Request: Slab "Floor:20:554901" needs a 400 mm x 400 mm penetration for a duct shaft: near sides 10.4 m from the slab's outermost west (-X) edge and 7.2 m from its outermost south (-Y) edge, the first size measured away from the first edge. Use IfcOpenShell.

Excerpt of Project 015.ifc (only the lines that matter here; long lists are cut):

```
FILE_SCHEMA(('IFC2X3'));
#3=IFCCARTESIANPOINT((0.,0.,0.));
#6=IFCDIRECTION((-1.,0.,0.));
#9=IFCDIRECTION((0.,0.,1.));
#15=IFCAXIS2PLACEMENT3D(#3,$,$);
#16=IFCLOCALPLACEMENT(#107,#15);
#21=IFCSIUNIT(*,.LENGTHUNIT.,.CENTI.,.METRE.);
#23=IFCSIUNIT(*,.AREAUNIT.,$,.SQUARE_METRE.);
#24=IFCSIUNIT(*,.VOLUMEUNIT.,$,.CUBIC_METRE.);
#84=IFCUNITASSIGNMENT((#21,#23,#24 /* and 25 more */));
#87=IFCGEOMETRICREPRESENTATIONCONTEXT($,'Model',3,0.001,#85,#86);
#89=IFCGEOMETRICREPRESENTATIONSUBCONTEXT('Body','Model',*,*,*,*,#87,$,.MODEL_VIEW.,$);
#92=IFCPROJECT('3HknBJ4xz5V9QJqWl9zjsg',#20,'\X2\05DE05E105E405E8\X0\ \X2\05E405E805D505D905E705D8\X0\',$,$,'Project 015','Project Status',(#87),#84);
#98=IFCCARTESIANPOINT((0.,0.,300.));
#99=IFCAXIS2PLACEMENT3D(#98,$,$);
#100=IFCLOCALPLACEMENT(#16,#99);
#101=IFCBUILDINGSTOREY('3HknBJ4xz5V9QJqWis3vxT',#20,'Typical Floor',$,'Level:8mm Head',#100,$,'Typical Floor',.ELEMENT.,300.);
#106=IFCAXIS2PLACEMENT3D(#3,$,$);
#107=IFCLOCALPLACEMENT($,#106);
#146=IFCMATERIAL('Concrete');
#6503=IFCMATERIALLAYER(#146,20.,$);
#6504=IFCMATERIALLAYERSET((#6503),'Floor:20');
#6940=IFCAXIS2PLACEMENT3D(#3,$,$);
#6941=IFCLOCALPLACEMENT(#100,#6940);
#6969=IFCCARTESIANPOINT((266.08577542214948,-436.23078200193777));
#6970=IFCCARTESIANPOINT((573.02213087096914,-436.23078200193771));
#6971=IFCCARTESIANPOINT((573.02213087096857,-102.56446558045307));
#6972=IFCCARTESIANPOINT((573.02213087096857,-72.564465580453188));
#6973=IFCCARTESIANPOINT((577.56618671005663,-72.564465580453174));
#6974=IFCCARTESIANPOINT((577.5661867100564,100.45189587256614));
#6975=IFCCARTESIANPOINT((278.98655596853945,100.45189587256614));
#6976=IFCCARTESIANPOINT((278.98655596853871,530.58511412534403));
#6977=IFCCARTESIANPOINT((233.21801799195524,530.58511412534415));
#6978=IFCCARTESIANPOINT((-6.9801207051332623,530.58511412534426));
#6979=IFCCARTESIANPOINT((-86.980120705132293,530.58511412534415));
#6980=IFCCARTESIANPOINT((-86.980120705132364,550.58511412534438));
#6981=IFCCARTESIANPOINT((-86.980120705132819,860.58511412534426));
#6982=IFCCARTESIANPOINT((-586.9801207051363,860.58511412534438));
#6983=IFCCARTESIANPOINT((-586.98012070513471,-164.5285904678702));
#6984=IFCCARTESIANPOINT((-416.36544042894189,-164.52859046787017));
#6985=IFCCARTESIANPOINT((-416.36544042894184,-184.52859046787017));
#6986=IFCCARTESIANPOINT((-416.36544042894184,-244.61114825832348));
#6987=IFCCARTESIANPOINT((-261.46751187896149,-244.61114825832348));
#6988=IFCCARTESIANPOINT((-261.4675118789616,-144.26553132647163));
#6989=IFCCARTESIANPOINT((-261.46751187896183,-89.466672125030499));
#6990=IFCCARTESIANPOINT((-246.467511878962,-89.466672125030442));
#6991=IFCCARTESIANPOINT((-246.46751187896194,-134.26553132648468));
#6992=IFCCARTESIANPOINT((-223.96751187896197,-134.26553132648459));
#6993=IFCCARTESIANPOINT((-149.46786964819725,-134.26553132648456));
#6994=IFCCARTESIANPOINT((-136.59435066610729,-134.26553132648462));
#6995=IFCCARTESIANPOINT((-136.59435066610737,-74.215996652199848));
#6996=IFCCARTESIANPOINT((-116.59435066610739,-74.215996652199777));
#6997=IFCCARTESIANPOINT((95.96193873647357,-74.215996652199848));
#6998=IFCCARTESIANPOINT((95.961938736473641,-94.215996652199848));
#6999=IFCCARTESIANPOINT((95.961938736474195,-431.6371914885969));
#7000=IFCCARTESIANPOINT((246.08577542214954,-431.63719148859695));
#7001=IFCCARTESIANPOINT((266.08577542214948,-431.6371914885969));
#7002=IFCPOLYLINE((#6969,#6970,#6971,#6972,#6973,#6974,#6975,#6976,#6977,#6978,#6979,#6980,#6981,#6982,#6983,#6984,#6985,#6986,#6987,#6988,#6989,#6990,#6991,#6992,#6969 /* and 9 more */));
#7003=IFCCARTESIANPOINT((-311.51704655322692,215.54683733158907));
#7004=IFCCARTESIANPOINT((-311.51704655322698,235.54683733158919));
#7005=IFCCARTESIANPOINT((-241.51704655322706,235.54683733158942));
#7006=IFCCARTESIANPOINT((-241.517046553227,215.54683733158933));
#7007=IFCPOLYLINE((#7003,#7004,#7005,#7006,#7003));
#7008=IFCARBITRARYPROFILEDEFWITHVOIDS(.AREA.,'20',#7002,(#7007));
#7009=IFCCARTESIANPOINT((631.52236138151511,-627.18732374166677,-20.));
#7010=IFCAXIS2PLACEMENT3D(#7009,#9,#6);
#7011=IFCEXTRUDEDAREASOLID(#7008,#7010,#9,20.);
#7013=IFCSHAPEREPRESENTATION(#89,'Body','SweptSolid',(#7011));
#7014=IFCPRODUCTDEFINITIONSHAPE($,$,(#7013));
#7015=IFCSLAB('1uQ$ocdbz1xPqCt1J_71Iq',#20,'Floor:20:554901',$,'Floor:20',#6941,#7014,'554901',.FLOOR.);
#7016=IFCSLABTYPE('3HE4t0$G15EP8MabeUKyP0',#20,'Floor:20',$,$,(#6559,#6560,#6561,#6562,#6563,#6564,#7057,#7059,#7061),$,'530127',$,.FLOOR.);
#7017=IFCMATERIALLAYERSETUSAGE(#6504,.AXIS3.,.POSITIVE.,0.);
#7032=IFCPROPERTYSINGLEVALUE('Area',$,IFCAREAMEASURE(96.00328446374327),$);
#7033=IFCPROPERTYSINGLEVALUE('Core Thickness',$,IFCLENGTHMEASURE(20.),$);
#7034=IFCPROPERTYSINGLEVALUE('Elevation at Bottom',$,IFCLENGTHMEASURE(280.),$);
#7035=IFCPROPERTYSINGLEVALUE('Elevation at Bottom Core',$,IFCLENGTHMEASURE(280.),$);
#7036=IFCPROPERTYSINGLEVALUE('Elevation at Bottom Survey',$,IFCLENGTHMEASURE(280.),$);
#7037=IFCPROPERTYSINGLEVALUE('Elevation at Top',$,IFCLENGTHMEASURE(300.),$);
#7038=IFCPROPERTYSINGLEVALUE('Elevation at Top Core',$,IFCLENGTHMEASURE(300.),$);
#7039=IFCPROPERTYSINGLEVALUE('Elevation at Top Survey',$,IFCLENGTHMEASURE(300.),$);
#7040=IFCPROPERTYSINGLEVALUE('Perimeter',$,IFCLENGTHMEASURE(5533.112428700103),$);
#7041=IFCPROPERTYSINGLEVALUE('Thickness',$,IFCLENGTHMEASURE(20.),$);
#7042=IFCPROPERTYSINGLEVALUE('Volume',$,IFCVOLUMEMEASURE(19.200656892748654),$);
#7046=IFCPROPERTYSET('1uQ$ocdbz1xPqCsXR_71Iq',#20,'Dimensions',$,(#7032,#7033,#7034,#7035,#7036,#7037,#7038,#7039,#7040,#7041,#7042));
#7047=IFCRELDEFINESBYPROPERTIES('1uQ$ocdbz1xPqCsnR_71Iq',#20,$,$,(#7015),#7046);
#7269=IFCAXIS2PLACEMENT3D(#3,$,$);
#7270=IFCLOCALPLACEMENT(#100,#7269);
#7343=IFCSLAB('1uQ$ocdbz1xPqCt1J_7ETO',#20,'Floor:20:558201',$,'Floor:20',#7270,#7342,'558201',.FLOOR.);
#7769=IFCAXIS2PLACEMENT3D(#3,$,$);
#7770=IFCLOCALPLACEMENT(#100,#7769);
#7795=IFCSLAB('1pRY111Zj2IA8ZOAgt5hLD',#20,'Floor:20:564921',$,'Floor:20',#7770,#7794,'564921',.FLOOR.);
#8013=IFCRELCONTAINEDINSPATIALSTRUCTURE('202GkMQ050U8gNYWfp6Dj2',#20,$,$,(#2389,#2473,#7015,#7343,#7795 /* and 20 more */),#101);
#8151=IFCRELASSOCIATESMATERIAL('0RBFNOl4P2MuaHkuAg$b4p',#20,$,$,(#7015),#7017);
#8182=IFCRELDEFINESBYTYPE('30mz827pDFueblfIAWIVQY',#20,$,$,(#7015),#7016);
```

```python
import numpy as np
import ifcopenshell
import ifcopenshell.api.feature
import ifcopenshell.api.geometry
import ifcopenshell.api.pset
import ifcopenshell.api.root
import ifcopenshell.geom
import ifcopenshell.util.element
import ifcopenshell.util.placement
import ifcopenshell.util.representation
import ifcopenshell.util.shape
import ifcopenshell.util.unit

model = ifcopenshell.open("Project 015.ifc")
unit_scale = ifcopenshell.util.unit.calculate_unit_scale(model)
area_scale = ifcopenshell.util.unit.calculate_unit_scale(model, "AREAUNIT")
volume_scale = ifcopenshell.util.unit.calculate_unit_scale(model, "VOLUMEUNIT")
settings = ifcopenshell.geom.settings()


def volume(element):
    """Net volume in cubic metres, openings subtracted."""
    shape = ifcopenshell.geom.create_shape(settings, element)
    return ifcopenshell.util.shape.get_volume(shape.geometry)


slab = model.by_id(7015)
before = volume(slab)

# Extent in the slab's own axes, in metres. The edges named are its -X and -Y sides.
slab_shape = ifcopenshell.geom.create_shape(settings, slab)
vertices = ifcopenshell.util.shape.get_vertices(slab_shape.geometry)
x_min, y_min, bottom = vertices.min(axis=0)
top = vertices[:, 2].max()

opening = ifcopenshell.api.root.create_entity(model, ifc_class="IfcOpeningElement", name="Duct shaft opening")
context = ifcopenshell.util.representation.get_context(model, "Model", "Body", "MODEL_VIEW")
width, depth = 0.4, 0.4
outline = [(0.0, 0.0), (width, 0.0), (width, depth), (0.0, depth), (0.0, 0.0)]
# Overshoot both faces by 50 mm so the cut is clean.
shape = ifcopenshell.api.geometry.add_slab_representation(
    model, context=context, depth=top - bottom + 0.1, polyline=outline
)
ifcopenshell.api.geometry.assign_representation(model, product=opening, representation=shape)

matrix = ifcopenshell.util.placement.get_local_placement(slab.ObjectPlacement)
matrix[:, 3] = matrix @ np.append(np.array([x_min + 10.4, y_min + 7.2, bottom - 0.05]) / unit_scale, 1.0)
ifcopenshell.api.geometry.edit_object_placement(model, product=opening, matrix=matrix, is_si=False)
ifcopenshell.api.feature.add_feature(model, feature=opening, element=slab)

after = volume(slab)

# Update the slab's stored quantities.
pset = model.by_id(ifcopenshell.util.element.get_pset(slab, "Dimensions", should_inherit=False)["id"])
ifcopenshell.api.pset.edit_pset(model, pset=pset, properties={
    "Area": model.create_entity("IfcAreaMeasure", after / (top - bottom) / area_scale),
    "Volume": model.create_entity("IfcVolumeMeasure", after / volume_scale),
})

print(f"slab volume {before:.3f} -> {after:.3f} m3")

model.write("Project 015-out.ifc")
```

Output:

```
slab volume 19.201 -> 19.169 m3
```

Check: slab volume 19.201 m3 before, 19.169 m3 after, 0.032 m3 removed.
